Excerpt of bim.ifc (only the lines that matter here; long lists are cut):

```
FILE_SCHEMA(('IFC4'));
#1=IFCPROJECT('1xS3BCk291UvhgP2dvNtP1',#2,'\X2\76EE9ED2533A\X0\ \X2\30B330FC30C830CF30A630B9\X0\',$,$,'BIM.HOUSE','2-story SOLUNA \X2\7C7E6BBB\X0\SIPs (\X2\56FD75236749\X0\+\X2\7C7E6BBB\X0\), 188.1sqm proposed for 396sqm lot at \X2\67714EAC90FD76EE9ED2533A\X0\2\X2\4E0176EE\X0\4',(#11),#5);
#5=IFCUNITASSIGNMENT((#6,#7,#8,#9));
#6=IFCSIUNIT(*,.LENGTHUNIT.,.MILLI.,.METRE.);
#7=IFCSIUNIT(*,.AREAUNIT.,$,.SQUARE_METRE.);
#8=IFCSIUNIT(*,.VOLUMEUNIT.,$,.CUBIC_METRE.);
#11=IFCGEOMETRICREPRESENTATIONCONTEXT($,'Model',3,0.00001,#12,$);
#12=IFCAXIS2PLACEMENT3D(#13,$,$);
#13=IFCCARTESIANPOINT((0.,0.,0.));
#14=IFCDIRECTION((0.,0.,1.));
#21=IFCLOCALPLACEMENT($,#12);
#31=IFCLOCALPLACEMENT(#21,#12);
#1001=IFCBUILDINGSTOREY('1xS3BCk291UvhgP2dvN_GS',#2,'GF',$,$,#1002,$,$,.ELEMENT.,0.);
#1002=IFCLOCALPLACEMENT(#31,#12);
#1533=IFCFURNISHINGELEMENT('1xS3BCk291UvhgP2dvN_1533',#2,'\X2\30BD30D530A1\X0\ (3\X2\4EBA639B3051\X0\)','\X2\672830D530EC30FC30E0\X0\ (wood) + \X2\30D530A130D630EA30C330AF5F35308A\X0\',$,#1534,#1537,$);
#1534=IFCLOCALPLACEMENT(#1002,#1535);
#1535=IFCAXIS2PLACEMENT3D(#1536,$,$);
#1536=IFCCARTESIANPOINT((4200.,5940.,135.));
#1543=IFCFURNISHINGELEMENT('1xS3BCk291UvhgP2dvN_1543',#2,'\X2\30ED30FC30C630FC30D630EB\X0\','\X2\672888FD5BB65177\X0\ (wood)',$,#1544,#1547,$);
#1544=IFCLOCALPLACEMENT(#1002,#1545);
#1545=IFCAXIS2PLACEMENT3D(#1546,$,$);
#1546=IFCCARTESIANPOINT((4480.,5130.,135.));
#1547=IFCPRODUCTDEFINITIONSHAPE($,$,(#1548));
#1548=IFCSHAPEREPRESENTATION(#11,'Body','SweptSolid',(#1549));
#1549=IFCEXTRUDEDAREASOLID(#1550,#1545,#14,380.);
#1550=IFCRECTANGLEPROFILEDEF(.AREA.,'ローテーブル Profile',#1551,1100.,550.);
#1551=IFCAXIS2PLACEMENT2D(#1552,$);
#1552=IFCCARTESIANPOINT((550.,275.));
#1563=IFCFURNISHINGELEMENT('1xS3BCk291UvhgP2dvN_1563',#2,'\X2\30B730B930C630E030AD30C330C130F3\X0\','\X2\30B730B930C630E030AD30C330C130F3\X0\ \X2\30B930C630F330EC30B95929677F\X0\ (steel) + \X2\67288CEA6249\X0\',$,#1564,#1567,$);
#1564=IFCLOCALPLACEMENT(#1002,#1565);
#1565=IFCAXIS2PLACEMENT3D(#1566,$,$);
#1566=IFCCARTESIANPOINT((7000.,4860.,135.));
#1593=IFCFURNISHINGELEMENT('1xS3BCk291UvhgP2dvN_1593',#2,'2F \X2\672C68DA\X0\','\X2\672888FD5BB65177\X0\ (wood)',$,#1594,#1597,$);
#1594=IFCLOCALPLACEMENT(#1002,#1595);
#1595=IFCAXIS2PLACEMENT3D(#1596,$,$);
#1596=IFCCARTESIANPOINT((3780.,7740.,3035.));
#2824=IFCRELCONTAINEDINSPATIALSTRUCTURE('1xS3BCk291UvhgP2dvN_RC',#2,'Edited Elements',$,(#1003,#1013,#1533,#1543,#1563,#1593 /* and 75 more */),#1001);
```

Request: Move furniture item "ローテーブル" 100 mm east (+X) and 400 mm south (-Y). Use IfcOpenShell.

```python
import ifcopenshell
import ifcopenshell.api.geometry
import ifcopenshell.util.placement

model = ifcopenshell.open("bim.ifc")

item = model.by_id(1543)
matrix = ifcopenshell.util.placement.get_local_placement(item.ObjectPlacement)
matrix[0, 3] += 100.0
matrix[1, 3] -= 400.0
ifcopenshell.api.geometry.edit_object_placement(model, product=item, matrix=matrix, is_si=False)

print(ifcopenshell.util.placement.get_local_placement(item.ObjectPlacement).round(3) + 0.0)

model.write("bim_v2.ifc")
```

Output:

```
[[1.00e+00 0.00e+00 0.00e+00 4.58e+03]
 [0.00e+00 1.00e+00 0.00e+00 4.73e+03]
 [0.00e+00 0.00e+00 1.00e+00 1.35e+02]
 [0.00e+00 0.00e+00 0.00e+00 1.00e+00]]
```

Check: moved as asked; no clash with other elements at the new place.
